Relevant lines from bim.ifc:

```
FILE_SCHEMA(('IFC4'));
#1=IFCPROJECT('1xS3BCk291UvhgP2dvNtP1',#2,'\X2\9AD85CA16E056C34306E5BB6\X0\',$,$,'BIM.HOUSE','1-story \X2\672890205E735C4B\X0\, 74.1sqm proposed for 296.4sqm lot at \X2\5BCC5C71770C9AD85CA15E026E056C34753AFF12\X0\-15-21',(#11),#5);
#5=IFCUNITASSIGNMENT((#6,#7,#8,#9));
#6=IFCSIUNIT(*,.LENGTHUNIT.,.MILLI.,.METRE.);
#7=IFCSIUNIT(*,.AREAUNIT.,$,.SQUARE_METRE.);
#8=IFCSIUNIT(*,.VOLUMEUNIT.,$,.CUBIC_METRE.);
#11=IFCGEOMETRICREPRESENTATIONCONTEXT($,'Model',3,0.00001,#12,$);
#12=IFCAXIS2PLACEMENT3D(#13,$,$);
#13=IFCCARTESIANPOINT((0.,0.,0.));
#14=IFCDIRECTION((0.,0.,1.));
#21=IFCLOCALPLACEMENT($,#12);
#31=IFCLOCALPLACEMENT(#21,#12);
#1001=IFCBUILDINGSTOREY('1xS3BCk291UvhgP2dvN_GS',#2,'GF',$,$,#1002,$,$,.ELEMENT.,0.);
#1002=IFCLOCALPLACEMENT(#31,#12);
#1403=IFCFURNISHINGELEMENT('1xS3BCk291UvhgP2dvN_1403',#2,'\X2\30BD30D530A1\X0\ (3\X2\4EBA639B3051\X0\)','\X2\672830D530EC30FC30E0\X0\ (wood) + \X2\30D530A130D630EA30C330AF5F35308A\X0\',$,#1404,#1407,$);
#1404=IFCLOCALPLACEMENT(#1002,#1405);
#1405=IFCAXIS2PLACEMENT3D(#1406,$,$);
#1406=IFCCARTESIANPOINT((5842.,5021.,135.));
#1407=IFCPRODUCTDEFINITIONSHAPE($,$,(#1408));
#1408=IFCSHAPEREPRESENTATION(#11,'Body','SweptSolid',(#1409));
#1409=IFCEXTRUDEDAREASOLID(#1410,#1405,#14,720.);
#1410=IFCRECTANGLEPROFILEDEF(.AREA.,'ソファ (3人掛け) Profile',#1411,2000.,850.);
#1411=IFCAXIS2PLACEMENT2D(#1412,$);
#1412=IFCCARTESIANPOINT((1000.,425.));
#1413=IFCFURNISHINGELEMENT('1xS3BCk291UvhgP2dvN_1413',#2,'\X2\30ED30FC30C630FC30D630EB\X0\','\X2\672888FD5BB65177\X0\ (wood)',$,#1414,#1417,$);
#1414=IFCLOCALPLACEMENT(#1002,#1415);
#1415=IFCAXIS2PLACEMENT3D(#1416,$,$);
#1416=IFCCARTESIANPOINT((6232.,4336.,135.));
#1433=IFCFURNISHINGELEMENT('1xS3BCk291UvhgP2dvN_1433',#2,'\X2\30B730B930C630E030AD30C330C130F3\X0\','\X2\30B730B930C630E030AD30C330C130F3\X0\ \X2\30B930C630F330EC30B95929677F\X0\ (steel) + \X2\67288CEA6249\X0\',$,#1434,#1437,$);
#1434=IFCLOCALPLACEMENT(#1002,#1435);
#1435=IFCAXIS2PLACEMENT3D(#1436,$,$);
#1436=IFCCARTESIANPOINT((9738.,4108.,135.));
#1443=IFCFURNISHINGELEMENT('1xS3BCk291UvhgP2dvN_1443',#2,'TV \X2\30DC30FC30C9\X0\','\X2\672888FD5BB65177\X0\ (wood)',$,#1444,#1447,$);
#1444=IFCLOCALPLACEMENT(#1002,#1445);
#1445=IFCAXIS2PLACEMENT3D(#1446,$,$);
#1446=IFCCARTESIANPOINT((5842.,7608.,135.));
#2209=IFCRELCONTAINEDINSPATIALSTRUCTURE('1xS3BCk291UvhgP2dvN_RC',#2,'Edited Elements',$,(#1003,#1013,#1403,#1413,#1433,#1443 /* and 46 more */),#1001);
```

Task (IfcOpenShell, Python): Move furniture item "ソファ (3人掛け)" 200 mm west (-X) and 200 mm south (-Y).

```python
import ifcopenshell
import ifcopenshell.api.geometry
import ifcopenshell.util.placement
import ifcopenshell.util.unit

model = ifcopenshell.open("bim.ifc")
unit_scale = ifcopenshell.util.unit.calculate_unit_scale(model)

item = model.by_guid("1xS3BCk291UvhgP2dvN_1403")
matrix = ifcopenshell.util.placement.get_local_placement(item.ObjectPlacement)
matrix[0, 3] -= 0.2 / unit_scale
matrix[1, 3] -= 0.2 / unit_scale
ifcopenshell.api.geometry.edit_object_placement(model, product=item, matrix=matrix, is_si=False)

print(ifcopenshell.util.placement.get_local_placement(item.ObjectPlacement).round(3) + 0.0)

model.write("bim-out.ifc")
```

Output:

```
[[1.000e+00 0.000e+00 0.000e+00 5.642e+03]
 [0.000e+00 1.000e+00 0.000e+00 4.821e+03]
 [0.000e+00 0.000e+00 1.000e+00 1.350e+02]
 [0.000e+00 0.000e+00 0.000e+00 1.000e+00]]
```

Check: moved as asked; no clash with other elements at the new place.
